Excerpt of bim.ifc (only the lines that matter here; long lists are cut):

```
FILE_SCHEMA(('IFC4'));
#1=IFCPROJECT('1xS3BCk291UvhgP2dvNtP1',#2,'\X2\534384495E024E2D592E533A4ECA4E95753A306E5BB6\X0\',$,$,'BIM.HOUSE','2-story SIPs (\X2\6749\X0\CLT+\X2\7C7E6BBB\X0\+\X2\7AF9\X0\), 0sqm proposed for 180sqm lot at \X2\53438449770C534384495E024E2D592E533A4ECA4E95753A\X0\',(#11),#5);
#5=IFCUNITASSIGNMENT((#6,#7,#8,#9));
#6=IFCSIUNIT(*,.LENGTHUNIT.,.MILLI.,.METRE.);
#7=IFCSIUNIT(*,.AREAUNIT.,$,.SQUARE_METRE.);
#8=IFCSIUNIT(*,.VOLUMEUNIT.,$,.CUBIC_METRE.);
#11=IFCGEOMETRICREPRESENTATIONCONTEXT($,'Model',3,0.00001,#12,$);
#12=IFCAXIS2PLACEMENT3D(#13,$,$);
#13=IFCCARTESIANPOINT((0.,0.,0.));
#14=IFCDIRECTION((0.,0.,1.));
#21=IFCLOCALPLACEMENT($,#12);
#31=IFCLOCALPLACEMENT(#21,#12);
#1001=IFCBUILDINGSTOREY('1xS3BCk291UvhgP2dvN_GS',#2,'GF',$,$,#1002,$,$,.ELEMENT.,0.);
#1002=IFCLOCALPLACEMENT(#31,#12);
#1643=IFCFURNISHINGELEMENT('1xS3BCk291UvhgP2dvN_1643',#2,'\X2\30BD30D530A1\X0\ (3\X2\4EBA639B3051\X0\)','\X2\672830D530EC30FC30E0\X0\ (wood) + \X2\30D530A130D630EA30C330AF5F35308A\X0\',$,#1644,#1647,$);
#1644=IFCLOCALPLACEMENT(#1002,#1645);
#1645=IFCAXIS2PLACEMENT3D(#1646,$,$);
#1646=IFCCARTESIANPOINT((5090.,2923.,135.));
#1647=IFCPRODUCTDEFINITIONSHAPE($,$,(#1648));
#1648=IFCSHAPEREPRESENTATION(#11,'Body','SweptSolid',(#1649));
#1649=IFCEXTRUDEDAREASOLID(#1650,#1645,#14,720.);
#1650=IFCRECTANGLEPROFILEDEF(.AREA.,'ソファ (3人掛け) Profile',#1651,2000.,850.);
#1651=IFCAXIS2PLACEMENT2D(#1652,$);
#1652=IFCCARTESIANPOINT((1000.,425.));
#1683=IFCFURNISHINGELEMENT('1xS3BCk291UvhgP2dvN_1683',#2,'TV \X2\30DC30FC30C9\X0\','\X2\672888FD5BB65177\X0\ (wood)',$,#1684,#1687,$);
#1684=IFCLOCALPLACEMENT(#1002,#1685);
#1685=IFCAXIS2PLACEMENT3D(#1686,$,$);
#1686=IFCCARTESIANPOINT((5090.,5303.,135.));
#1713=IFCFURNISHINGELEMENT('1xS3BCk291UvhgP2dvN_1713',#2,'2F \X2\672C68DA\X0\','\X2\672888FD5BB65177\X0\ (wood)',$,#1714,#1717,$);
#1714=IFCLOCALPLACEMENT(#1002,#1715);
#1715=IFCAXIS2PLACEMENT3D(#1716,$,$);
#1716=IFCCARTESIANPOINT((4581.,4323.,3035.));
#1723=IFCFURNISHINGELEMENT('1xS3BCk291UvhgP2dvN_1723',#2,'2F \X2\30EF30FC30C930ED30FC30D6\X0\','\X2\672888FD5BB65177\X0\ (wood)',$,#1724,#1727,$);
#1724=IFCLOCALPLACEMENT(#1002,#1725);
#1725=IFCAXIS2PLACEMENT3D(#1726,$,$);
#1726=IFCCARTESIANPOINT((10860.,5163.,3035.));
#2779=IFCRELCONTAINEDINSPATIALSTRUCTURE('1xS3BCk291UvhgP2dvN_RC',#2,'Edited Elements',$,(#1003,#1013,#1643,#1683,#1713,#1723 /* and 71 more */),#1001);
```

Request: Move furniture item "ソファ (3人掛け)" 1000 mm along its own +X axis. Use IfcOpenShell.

```python
import ifcopenshell
import ifcopenshell.api.geometry
import ifcopenshell.util.placement
import ifcopenshell.util.unit

model = ifcopenshell.open("bim.ifc")
unit_scale = ifcopenshell.util.unit.calculate_unit_scale(model)

item = model.by_guid("1xS3BCk291UvhgP2dvN_1643")
matrix = ifcopenshell.util.placement.get_local_placement(item.ObjectPlacement)
matrix[:3, 3] += matrix[:3, 0] * 1 / unit_scale
ifcopenshell.api.geometry.edit_object_placement(model, product=item, matrix=matrix, is_si=False)

print(ifcopenshell.util.placement.get_local_placement(item.ObjectPlacement).round(3) + 0.0)

model.write("bim_updated.ifc")
```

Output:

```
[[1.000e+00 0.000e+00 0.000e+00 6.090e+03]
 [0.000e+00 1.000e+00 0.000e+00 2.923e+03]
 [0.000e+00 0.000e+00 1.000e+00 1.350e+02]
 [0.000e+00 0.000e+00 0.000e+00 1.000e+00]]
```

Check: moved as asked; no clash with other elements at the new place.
